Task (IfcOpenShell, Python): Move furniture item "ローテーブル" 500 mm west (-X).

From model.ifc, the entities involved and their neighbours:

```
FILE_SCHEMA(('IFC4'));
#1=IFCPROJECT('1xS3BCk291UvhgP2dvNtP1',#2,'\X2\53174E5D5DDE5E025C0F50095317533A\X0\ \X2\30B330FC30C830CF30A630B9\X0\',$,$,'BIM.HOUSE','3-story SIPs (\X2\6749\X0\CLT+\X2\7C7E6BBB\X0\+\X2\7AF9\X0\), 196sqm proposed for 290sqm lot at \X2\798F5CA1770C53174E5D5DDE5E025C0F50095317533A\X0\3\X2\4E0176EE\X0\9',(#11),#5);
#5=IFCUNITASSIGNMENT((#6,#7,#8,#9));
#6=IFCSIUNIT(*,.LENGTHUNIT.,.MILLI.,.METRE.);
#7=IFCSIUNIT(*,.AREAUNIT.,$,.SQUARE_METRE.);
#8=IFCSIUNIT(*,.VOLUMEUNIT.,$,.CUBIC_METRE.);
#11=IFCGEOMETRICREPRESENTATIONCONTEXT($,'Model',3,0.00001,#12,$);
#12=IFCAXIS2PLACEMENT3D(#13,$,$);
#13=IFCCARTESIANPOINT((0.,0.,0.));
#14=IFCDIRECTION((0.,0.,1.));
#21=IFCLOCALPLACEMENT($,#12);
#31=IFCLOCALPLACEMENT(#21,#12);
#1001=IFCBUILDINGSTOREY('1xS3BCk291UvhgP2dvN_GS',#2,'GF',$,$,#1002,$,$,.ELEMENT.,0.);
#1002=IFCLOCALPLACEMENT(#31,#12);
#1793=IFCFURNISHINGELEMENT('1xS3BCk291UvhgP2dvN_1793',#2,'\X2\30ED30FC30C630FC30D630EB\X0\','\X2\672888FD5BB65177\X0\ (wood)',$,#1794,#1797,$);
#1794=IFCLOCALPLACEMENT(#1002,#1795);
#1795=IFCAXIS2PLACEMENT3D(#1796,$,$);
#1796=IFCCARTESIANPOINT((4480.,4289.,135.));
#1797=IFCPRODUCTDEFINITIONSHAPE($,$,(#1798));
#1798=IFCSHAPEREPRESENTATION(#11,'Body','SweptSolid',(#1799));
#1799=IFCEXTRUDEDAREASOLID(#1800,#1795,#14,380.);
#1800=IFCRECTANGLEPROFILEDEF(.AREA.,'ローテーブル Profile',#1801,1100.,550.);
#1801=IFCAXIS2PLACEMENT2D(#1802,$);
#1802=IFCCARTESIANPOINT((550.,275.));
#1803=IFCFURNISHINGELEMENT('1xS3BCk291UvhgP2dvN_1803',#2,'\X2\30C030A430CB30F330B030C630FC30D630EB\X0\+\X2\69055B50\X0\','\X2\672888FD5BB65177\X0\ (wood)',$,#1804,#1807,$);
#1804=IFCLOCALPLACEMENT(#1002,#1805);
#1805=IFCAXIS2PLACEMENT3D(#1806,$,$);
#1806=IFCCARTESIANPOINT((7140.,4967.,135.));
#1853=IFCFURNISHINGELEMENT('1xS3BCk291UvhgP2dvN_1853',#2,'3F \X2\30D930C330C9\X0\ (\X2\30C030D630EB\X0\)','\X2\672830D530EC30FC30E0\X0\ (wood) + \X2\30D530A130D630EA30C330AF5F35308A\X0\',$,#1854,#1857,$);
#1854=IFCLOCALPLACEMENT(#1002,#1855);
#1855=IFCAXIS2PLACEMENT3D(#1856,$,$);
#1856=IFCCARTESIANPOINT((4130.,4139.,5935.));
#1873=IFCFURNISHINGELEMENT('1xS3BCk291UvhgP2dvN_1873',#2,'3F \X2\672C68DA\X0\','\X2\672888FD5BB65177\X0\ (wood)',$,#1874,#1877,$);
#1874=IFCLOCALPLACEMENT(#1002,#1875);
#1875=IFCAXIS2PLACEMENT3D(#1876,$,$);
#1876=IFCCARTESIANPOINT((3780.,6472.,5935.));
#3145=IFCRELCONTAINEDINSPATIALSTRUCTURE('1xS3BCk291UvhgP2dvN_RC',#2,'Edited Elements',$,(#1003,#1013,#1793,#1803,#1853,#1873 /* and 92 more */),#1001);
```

```python
import ifcopenshell
import ifcopenshell.api.geometry
import ifcopenshell.util.placement

model = ifcopenshell.open("model.ifc")

item = model.by_id(1793)
matrix = ifcopenshell.util.placement.get_local_placement(item.ObjectPlacement)
matrix[0, 3] -= 500.0
ifcopenshell.api.geometry.edit_object_placement(model, product=item, matrix=matrix, is_si=False)

print(ifcopenshell.util.placement.get_local_placement(item.ObjectPlacement).round(3) + 0.0)

model.write("model_updated.ifc")
```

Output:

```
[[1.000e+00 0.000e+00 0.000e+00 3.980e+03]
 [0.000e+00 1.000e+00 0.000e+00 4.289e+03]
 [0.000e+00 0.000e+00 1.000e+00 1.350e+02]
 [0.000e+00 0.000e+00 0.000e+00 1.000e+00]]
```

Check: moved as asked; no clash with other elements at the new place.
